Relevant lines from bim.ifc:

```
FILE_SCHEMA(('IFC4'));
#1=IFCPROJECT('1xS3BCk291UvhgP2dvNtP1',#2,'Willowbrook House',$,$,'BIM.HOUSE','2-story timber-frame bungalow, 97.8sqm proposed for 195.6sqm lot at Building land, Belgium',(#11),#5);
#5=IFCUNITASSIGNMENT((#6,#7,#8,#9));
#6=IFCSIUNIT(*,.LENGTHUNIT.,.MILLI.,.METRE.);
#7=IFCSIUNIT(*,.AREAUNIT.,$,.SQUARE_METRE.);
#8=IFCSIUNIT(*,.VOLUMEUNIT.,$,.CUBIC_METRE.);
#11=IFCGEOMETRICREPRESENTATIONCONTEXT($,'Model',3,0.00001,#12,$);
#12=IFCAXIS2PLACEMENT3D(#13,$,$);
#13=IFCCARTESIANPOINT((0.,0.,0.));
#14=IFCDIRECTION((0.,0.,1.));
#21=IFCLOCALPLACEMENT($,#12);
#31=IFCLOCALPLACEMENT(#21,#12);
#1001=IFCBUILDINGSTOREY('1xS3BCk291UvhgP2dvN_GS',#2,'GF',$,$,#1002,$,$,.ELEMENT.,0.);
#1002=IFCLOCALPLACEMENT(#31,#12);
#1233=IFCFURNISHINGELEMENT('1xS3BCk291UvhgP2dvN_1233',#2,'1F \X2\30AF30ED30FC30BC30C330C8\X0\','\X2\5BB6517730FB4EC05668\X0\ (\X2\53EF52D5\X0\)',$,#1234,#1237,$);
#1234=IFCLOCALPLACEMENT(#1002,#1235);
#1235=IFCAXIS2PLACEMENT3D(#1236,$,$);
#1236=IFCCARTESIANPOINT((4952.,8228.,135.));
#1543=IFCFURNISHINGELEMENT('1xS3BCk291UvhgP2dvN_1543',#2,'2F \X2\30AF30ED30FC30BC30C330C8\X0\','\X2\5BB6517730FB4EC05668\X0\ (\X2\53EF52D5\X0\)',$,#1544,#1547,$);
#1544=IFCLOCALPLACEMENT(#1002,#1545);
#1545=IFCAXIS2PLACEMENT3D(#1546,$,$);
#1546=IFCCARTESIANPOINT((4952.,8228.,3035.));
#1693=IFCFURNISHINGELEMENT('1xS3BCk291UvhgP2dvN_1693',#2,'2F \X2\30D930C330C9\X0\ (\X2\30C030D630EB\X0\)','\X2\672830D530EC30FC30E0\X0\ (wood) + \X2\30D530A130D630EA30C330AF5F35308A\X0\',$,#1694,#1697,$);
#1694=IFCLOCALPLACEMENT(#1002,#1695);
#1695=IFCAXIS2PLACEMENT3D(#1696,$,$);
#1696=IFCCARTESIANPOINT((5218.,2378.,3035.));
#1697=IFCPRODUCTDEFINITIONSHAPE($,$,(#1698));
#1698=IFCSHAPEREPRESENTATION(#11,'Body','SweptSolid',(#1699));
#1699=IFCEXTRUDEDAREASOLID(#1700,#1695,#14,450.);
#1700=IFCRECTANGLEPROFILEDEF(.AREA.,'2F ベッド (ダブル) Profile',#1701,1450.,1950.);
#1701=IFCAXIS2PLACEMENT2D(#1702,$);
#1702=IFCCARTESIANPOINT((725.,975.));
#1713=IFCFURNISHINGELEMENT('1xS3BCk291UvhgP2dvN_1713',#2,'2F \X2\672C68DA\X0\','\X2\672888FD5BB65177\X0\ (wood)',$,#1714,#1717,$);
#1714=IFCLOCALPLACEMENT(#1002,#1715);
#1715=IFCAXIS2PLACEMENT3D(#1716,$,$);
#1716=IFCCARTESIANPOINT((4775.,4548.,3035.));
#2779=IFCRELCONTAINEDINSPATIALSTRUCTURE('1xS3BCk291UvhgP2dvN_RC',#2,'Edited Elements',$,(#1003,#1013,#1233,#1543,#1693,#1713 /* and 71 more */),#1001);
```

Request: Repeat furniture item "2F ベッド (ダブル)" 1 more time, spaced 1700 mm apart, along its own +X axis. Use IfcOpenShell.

```python
import ifcopenshell
import ifcopenshell.api.geometry
import ifcopenshell.api.root
import ifcopenshell.util.element
import ifcopenshell.util.placement
import ifcopenshell.util.unit

model = ifcopenshell.open("bim.ifc")
unit_scale = ifcopenshell.util.unit.calculate_unit_scale(model)


def reuse_history(source, copy):
    """copy_class also copies each property set's owner history, people and application; keep the originals."""
    for rel in copy.IsDefinedBy:
        if rel.is_a("IfcRelDefinesByProperties") and (history := rel.RelatingPropertyDefinition.OwnerHistory):
            rel.RelatingPropertyDefinition.OwnerHistory = source.OwnerHistory
            ifcopenshell.util.element.remove_deep2(model, history)


source = model.by_id(1693)
base = ifcopenshell.util.placement.get_local_placement(source.ObjectPlacement)
step = base[:3, 0] * 1.7 / unit_scale

for i in range(1, 2):
    copy = ifcopenshell.api.root.copy_class(model, product=source)
    copy.Representation = ifcopenshell.util.element.copy_deep(
        model, source.Representation, exclude=["IfcGeometricRepresentationContext", "IfcRepresentationMap"]
    )
    reuse_history(source, copy)
    matrix = base.copy()
    matrix[:3, 3] += i * step
    print("added at", matrix[:3, 3].round(3) + 0.0)
    ifcopenshell.api.geometry.edit_object_placement(model, product=copy, matrix=matrix, is_si=False)

model.write("bim_updated.ifc")
```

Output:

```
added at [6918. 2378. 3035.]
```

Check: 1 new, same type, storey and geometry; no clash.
